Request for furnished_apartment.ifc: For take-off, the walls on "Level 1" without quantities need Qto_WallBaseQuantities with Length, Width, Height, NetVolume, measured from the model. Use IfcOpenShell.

First a look at what the model holds.

```python
import ifcopenshell
import ifcopenshell.util.element
import ifcopenshell.util.unit

model = ifcopenshell.open("furnished_apartment.ifc")
print(model.schema)
for unit_type in ("LENGTHUNIT", "AREAUNIT", "VOLUMEUNIT"):
    print(unit_type, ifcopenshell.util.unit.calculate_unit_scale(model, unit_type))
storey = next(s for s in model.by_type("IfcBuildingStorey") if s.Name == "Level 1")
walls = [e for e in ifcopenshell.util.element.get_decomposition(storey) if e.is_a("IfcWall")]
for e in sorted(walls, key=lambda e: e.id()):
    print(e.id(), e.is_a(), e.Name, list(ifcopenshell.util.element.get_psets(e, qtos_only=True)), sep=" | ")
```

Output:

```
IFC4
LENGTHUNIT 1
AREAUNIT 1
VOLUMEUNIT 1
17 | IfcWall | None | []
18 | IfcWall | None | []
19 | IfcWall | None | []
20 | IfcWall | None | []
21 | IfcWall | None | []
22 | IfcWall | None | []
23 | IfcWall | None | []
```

```python
import ifcopenshell
import ifcopenshell.api.pset
import ifcopenshell.geom
import ifcopenshell.util.element
import ifcopenshell.util.shape
import ifcopenshell.util.unit

model = ifcopenshell.open("furnished_apartment.ifc")
unit_scale = ifcopenshell.util.unit.calculate_unit_scale(model)
volume_scale = ifcopenshell.util.unit.calculate_unit_scale(model, "VOLUMEUNIT")
settings = ifcopenshell.geom.settings()

storey = next(s for s in model.by_type("IfcBuildingStorey") if s.Name == "Level 1")
walls = [e for e in ifcopenshell.util.element.get_decomposition(storey) if e.is_a("IfcWall")]

for e in sorted(walls, key=lambda e: e.id()):
    if ifcopenshell.util.element.get_psets(e, qtos_only=True, should_inherit=False):
        continue
    # Geometry comes back in metres, in the element's own axes.
    shape = ifcopenshell.geom.create_shape(settings, e)
    values = {
        "Length": ifcopenshell.util.shape.get_x(shape.geometry) / unit_scale,
        "Width": ifcopenshell.util.shape.get_y(shape.geometry) / unit_scale,
        "Height": ifcopenshell.util.shape.get_z(shape.geometry) / unit_scale,
        "NetVolume": ifcopenshell.util.shape.get_volume(shape.geometry) / volume_scale,
    }
    qto = ifcopenshell.api.pset.add_qto(model, product=e, name="Qto_WallBaseQuantities")
    ifcopenshell.api.pset.edit_qto(model, qto=qto, properties=values)
    print(e.id(), {k: round(v, 3) for k, v in values.items()})

model.write("furnished_apartment_rev.ifc")
```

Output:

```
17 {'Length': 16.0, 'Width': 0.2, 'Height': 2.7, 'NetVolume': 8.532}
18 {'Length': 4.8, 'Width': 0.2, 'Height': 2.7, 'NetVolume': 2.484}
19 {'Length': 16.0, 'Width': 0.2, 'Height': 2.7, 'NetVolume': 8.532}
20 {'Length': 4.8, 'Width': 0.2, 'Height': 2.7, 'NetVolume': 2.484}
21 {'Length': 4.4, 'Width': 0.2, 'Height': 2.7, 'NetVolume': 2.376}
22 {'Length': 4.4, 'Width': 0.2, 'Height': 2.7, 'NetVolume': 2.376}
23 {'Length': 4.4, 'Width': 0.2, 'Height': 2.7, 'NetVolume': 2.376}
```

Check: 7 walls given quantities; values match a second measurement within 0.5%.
